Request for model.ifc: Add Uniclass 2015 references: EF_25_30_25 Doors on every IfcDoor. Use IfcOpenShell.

First a look at what the model holds.

```python
import ifcopenshell

model = ifcopenshell.open("model.ifc")
print(model.schema)
print("classifications:", [c.Name for c in model.by_type("IfcClassification")])
for ifc_class in ("IfcDoor", "IfcRoof", "IfcStair", "IfcWall", "IfcWindow"):
    print(ifc_class, len(model.by_type(ifc_class)))
```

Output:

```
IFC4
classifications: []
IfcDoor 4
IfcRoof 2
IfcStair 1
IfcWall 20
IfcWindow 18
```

```python
import ifcopenshell
import ifcopenshell.api.classification

model = ifcopenshell.open("model.ifc")

system = ifcopenshell.api.classification.add_classification(model, classification="Uniclass 2015")

codes = {
    "IfcDoor": ("EF_25_30_25", "Doors"),
}
for ifc_class, (code, name) in codes.items():
    products = model.by_type(ifc_class)
    ifcopenshell.api.classification.add_reference(
        model, products=products, classification=system, identification=code, name=name
    )
    print(code, len(products))

model.write("model_v2.ifc")
```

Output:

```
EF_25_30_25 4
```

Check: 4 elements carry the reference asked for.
